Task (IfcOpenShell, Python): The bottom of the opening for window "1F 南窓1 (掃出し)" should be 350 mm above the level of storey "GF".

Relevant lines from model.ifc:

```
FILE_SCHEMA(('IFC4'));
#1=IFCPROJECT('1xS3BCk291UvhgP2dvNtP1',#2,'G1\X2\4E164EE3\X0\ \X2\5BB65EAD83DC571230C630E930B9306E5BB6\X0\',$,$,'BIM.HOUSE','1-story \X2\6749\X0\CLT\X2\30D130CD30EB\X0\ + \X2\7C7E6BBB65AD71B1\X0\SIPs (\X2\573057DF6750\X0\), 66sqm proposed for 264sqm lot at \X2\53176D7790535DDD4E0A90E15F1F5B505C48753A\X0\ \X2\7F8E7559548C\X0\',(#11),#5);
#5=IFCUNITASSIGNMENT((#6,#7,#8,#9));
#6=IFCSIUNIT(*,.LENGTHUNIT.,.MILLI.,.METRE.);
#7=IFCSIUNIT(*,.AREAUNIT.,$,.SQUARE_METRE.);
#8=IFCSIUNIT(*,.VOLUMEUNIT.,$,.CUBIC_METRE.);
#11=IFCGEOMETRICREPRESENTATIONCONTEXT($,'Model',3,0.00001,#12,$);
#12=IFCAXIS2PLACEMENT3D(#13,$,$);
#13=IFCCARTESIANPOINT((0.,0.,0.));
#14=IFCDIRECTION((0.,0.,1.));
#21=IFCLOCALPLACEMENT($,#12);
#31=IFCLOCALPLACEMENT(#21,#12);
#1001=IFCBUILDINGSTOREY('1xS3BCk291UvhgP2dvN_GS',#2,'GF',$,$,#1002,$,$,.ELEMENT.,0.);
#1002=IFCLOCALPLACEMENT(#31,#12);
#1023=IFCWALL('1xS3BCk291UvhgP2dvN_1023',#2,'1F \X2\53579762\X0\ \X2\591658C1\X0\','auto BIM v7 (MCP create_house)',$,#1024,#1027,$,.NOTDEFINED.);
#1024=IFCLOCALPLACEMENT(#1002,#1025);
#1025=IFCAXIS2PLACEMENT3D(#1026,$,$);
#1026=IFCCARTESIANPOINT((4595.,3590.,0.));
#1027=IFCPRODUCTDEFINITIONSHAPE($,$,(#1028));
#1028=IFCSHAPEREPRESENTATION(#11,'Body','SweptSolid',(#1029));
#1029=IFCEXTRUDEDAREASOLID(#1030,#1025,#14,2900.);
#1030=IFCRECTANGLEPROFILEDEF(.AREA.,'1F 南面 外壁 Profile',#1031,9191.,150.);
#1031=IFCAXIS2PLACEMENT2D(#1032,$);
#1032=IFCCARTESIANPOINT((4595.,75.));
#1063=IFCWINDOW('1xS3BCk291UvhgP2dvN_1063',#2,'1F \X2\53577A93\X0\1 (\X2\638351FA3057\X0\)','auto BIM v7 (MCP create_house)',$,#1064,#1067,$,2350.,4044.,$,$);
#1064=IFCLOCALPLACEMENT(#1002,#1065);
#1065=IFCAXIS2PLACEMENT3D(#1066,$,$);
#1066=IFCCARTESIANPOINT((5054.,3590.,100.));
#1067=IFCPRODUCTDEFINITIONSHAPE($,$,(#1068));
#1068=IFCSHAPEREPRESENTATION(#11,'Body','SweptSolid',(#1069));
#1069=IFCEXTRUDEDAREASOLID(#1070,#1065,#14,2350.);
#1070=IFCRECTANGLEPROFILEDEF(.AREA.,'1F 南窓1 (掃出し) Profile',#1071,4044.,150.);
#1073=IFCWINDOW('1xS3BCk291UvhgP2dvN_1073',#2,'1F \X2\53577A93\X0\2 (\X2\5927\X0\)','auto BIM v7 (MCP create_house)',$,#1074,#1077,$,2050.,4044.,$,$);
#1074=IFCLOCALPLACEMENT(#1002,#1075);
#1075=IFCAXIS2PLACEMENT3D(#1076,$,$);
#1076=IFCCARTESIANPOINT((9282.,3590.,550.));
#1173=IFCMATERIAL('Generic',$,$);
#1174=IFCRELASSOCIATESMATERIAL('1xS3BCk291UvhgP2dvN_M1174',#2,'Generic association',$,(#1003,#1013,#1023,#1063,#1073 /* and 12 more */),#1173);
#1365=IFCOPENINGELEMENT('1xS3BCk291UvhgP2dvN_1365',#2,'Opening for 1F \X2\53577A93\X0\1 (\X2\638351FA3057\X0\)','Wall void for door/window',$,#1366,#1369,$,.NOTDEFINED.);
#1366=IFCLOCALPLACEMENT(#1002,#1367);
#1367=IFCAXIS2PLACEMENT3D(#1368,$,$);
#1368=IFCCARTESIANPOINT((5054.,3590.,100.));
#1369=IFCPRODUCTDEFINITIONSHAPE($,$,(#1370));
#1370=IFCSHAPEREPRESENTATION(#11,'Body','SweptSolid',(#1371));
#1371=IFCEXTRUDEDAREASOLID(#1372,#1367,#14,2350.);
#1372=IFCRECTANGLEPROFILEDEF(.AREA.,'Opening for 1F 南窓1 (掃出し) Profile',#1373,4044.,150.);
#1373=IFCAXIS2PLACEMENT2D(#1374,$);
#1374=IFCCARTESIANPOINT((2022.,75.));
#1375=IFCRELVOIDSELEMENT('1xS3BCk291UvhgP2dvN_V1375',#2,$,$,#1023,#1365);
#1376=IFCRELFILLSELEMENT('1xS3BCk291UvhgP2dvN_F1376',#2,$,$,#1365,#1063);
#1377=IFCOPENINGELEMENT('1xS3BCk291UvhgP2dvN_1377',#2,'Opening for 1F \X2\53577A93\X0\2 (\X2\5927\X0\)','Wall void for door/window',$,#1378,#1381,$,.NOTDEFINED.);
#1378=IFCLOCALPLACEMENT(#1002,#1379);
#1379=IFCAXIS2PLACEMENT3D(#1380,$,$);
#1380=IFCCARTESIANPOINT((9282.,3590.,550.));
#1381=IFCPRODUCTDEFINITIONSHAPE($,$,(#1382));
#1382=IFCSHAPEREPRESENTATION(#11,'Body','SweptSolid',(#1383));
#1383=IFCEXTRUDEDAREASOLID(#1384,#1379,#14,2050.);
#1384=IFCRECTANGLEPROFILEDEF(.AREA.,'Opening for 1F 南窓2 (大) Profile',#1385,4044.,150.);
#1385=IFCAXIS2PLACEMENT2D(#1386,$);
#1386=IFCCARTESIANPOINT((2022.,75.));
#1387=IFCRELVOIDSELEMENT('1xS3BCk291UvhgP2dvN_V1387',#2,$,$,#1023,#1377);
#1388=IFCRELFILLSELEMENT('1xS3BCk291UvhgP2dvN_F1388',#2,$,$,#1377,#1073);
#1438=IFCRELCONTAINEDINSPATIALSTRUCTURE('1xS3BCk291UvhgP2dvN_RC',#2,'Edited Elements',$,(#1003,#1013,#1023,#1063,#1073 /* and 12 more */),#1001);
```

```python
import numpy as np
import ifcopenshell
import ifcopenshell.api.geometry
import ifcopenshell.geom
import ifcopenshell.util.element
import ifcopenshell.util.placement
import ifcopenshell.util.shape
import ifcopenshell.util.unit

model = ifcopenshell.open("model.ifc")
unit_scale = ifcopenshell.util.unit.calculate_unit_scale(model)

window = model.by_guid("1xS3BCk291UvhgP2dvN_1063")
opening = window.FillsVoids[0].RelatingOpeningElement
storey = ifcopenshell.util.element.get_container(window, ifc_class="IfcBuildingStorey")
level = ifcopenshell.util.placement.get_local_placement(storey.ObjectPlacement)[2, 3]

# The opening's origin need not be at the sill, so measure its lowest point.
shape = ifcopenshell.geom.create_shape(ifcopenshell.geom.settings(), opening)
bottom = ifcopenshell.util.shape.get_shape_bottom_elevation(shape, shape.geometry) / unit_scale
dz = level + 0.35 / unit_scale - bottom

shift = np.array([0.0, 0.0, dz])
# The window is not placed relative to its opening, so move both.
for product in (opening, window):
    matrix = ifcopenshell.util.placement.get_local_placement(product.ObjectPlacement)
    matrix[:3, 3] += shift
    ifcopenshell.api.geometry.edit_object_placement(model, product=product, matrix=matrix, is_si=False)

print(f"moved by {dz * unit_scale:+.3f} m")

model.write("model_edited.ifc")
```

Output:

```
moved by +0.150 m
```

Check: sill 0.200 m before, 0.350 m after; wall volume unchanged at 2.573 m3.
